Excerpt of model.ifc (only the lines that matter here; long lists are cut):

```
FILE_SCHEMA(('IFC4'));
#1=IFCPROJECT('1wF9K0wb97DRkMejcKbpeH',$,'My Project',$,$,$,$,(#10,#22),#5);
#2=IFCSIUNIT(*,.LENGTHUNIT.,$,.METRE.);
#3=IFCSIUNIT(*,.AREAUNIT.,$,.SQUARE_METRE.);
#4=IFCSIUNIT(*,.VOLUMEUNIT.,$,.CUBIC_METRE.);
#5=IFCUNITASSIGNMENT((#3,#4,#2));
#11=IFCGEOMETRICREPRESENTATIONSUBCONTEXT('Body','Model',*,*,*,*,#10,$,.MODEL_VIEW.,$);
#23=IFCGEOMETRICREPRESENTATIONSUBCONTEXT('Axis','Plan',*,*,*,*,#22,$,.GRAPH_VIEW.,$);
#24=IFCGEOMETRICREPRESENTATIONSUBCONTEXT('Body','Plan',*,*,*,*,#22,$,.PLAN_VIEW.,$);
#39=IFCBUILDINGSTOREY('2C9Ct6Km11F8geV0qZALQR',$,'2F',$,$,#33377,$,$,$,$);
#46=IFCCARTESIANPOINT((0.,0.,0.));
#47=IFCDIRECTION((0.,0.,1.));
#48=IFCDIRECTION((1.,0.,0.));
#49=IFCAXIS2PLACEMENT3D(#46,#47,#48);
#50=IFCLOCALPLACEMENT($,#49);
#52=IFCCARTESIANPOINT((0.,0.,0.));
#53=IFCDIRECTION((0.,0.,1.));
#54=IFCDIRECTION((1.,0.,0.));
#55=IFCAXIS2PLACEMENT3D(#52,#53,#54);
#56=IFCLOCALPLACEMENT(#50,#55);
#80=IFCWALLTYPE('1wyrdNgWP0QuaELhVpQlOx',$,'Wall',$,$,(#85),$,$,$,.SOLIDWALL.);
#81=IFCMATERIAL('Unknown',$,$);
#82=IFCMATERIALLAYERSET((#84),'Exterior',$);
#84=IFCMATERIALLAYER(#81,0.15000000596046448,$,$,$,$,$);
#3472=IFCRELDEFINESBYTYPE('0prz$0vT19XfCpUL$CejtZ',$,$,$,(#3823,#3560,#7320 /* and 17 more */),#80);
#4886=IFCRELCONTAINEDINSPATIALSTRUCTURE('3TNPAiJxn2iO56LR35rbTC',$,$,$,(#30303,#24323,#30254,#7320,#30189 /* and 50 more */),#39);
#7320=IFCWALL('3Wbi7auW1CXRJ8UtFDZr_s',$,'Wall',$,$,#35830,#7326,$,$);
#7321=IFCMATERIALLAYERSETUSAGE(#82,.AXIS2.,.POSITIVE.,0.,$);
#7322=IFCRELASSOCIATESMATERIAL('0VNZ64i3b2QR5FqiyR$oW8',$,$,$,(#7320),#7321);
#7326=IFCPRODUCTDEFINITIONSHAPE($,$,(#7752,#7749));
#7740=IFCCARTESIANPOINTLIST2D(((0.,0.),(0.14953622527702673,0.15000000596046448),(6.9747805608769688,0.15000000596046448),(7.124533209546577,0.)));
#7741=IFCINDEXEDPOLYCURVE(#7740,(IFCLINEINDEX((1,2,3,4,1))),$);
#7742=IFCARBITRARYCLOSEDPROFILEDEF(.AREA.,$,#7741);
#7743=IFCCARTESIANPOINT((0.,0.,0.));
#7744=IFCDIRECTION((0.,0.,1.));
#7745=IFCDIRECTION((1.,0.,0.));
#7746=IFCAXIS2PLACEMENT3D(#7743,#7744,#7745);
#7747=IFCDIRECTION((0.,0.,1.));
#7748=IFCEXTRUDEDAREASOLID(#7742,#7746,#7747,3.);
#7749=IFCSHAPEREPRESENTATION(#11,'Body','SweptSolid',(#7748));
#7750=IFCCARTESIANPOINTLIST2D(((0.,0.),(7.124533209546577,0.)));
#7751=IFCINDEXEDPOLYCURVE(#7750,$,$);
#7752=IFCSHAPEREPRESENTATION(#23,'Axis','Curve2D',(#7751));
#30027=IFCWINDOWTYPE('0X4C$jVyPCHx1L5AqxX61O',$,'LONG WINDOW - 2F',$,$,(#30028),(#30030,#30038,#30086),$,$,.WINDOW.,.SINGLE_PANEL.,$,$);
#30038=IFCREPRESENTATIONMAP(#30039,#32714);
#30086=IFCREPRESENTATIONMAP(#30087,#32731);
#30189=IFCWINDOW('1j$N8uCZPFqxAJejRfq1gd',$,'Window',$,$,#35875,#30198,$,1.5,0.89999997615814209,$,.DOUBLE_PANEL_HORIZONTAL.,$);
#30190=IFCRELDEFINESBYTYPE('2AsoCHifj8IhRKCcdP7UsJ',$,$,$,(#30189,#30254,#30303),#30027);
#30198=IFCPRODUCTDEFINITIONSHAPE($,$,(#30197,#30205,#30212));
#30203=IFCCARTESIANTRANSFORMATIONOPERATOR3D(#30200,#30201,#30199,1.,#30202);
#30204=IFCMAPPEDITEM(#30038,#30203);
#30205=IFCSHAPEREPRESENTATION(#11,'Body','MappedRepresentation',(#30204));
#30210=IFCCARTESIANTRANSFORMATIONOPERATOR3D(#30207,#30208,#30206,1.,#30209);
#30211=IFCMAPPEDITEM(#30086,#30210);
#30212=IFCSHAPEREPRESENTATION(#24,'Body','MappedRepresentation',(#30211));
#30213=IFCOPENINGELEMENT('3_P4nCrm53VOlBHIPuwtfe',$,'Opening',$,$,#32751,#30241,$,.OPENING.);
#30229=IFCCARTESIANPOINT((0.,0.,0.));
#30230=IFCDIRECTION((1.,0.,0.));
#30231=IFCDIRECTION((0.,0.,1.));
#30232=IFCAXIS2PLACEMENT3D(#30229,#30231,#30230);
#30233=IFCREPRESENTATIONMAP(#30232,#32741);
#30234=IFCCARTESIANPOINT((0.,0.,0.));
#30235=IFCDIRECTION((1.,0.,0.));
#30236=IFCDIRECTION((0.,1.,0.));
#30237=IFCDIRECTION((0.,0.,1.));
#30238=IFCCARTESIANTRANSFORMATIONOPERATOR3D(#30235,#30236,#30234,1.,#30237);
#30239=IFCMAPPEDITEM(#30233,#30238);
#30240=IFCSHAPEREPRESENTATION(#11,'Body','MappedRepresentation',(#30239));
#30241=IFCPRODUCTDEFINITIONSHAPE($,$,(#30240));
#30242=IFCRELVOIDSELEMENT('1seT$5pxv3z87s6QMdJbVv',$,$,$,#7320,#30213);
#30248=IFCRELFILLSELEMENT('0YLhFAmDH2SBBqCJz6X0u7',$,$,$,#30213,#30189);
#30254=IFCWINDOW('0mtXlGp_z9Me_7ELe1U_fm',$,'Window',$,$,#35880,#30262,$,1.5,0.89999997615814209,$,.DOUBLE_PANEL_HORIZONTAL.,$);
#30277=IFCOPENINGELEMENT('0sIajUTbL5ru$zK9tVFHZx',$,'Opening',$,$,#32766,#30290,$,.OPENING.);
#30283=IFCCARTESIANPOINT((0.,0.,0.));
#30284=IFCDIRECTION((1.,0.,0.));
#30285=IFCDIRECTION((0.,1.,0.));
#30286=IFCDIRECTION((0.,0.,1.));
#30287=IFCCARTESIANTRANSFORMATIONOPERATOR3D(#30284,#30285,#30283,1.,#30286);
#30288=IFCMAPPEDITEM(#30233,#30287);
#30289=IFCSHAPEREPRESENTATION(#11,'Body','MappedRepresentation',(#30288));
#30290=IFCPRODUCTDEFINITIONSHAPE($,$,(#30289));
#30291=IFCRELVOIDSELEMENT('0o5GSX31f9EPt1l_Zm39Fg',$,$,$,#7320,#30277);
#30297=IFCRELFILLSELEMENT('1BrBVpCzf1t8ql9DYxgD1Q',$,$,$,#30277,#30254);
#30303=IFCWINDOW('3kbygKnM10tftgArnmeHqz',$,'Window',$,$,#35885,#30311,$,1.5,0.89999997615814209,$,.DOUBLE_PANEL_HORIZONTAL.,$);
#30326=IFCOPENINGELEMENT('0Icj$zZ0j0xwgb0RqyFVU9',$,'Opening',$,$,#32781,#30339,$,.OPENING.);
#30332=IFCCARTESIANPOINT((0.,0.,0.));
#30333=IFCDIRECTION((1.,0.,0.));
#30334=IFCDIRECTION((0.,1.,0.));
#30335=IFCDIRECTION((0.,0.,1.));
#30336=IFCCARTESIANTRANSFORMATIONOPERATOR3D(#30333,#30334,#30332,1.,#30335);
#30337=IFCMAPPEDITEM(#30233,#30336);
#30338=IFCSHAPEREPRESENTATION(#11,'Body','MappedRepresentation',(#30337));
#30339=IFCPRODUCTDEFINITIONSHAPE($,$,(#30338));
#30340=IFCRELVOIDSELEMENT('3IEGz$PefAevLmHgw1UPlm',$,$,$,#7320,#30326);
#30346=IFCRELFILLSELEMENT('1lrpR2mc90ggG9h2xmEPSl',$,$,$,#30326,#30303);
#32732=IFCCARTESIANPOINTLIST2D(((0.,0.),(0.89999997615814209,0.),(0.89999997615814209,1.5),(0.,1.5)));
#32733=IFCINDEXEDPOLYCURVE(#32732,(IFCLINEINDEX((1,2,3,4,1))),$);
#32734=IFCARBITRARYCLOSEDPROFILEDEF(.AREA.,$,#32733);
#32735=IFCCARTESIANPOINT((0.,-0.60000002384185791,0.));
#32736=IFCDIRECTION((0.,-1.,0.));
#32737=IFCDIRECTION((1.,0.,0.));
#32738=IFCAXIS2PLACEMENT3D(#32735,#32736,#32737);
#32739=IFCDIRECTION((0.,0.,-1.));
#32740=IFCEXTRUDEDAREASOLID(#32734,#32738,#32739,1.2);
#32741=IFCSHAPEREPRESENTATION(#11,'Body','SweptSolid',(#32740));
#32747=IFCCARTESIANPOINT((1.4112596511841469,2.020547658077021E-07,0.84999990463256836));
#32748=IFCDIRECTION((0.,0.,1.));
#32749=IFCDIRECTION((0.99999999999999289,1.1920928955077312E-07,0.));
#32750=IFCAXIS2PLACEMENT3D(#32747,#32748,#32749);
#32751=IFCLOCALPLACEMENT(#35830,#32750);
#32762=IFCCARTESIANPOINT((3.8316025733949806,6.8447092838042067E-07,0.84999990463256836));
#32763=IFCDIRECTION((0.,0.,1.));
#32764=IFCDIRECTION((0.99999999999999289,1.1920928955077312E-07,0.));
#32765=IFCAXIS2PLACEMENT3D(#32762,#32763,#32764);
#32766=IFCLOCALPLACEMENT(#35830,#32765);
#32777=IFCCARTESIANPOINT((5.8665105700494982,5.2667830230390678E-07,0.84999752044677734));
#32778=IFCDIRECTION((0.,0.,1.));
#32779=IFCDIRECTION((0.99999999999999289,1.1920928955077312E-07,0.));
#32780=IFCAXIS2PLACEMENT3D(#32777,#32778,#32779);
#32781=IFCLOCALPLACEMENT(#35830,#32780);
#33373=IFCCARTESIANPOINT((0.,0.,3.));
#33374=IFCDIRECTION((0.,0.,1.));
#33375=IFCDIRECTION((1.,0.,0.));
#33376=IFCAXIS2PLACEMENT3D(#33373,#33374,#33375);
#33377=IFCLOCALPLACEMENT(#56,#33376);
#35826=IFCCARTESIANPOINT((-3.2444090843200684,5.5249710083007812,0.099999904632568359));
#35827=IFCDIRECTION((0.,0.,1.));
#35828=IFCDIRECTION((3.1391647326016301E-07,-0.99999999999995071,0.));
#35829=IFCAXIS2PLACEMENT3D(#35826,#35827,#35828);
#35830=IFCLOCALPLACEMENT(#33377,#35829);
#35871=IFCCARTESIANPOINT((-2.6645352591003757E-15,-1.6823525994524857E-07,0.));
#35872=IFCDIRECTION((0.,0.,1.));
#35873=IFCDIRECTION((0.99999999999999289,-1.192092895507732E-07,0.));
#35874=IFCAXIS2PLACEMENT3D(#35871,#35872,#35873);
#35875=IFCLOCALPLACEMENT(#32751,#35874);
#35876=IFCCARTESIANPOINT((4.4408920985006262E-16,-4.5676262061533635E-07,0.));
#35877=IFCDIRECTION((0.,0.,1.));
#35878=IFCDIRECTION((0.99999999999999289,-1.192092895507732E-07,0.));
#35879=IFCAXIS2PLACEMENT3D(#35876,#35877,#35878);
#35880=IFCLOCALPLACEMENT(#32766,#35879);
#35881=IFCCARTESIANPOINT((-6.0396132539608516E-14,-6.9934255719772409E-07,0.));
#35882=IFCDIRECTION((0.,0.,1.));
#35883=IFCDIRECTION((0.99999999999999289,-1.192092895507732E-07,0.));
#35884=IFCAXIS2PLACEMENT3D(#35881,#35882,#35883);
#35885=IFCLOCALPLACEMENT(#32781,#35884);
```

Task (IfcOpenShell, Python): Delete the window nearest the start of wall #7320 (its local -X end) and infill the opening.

```python
import ifcopenshell
import ifcopenshell.api.feature
import ifcopenshell.api.root
import ifcopenshell.geom
import ifcopenshell.util.shape

model = ifcopenshell.open("model.ifc")
settings = ifcopenshell.geom.settings()


def volume(element):
    """Net volume in cubic metres, openings subtracted."""
    shape = ifcopenshell.geom.create_shape(settings, element)
    return ifcopenshell.util.shape.get_volume(shape.geometry)


window = model.by_id(30189)
opening = window.FillsVoids[0].RelatingOpeningElement
wall = opening.VoidsElements[0].RelatingBuildingElement
before = volume(wall)

ifcopenshell.api.root.remove_product(model, product=window)
ifcopenshell.api.feature.remove_feature(model, feature=opening)

after = volume(wall)

print(f"wall volume {before:.3f} -> {after:.3f} m3")

model.write("model-out.ifc")
```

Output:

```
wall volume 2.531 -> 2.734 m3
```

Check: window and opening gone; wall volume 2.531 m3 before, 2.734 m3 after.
